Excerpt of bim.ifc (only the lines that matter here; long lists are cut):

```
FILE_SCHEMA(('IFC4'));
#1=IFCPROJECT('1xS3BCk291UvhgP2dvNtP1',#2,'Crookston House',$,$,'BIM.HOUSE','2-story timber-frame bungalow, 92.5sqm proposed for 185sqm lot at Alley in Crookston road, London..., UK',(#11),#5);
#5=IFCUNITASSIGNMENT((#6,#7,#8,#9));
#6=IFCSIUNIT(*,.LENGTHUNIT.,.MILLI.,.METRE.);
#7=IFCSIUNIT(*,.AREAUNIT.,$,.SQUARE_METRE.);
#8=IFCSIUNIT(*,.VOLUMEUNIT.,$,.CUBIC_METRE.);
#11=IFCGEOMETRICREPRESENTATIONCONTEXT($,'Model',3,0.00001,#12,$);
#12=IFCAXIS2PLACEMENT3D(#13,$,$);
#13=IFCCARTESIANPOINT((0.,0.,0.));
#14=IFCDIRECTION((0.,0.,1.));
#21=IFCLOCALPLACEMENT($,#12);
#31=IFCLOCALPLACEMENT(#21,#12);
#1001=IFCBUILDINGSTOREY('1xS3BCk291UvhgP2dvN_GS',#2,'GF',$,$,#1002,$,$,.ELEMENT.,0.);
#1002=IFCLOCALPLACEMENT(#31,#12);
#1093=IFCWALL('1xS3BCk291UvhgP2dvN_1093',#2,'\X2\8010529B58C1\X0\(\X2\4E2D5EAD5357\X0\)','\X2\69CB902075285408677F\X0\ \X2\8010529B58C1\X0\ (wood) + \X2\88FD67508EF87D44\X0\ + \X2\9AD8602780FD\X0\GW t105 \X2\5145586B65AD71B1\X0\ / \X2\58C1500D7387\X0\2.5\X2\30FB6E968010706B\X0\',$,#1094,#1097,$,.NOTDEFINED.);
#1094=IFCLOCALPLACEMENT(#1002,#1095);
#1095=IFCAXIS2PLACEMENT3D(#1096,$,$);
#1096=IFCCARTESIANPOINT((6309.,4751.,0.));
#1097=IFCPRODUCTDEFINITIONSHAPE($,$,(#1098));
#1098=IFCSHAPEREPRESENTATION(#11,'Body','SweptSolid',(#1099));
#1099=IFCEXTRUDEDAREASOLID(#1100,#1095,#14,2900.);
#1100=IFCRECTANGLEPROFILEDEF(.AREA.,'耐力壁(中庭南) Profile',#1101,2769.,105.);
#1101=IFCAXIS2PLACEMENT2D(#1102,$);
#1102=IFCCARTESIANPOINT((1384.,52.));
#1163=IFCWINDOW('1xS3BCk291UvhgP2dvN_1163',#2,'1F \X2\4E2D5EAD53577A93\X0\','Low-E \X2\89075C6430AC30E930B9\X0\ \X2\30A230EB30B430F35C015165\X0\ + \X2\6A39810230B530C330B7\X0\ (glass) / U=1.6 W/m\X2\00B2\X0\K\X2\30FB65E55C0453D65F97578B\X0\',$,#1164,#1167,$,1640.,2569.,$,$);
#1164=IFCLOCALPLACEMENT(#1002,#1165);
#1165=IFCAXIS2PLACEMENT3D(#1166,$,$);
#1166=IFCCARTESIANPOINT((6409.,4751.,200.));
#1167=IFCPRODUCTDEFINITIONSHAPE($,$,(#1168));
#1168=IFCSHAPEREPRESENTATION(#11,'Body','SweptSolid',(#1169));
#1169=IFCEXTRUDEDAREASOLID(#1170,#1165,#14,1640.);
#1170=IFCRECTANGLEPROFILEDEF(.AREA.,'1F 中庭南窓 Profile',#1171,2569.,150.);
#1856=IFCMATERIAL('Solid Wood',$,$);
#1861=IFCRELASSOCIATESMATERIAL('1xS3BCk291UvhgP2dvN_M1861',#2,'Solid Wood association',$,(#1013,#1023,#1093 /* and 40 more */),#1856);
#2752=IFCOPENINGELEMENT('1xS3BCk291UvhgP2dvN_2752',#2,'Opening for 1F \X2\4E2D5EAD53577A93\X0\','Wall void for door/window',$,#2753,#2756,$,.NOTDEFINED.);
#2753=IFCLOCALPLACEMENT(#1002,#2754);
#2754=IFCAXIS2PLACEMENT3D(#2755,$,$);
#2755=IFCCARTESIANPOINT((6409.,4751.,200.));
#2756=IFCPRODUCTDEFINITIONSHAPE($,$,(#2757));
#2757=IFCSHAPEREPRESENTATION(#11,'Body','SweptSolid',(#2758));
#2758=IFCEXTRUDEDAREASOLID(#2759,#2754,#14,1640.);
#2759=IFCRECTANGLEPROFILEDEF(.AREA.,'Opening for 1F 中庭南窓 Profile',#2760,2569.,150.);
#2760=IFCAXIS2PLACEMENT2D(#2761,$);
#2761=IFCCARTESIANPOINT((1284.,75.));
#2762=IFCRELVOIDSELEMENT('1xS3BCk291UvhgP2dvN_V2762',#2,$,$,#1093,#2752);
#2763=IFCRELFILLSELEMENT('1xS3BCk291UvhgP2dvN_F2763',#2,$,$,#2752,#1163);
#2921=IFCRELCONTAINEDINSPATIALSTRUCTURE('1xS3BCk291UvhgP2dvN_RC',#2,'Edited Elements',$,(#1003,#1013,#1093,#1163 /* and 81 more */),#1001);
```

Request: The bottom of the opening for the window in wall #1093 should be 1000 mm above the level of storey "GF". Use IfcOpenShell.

```python
import numpy as np
import ifcopenshell
import ifcopenshell.api.geometry
import ifcopenshell.geom
import ifcopenshell.util.element
import ifcopenshell.util.placement
import ifcopenshell.util.shape
import ifcopenshell.util.unit

model = ifcopenshell.open("bim.ifc")
unit_scale = ifcopenshell.util.unit.calculate_unit_scale(model)

window = model.by_id(1163)
opening = window.FillsVoids[0].RelatingOpeningElement
storey = ifcopenshell.util.element.get_container(window, ifc_class="IfcBuildingStorey")
level = ifcopenshell.util.placement.get_local_placement(storey.ObjectPlacement)[2, 3]

# The opening's origin need not be at the sill, so measure its lowest point.
shape = ifcopenshell.geom.create_shape(ifcopenshell.geom.settings(), opening)
bottom = ifcopenshell.util.shape.get_shape_bottom_elevation(shape, shape.geometry) / unit_scale
dz = level + 1 / unit_scale - bottom

shift = np.array([0.0, 0.0, dz])
# The window is not placed relative to its opening, so move both.
for product in (opening, window):
    matrix = ifcopenshell.util.placement.get_local_placement(product.ObjectPlacement)
    matrix[:3, 3] += shift
    ifcopenshell.api.geometry.edit_object_placement(model, product=product, matrix=matrix, is_si=False)

print(f"moved by {dz * unit_scale:+.3f} m")

model.write("bim_rev.ifc")
```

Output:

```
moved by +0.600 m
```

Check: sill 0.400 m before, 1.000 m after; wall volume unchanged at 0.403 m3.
